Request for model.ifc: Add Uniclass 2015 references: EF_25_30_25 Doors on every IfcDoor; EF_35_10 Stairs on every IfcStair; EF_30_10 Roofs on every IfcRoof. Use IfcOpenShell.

First a look at what the model holds.

```python
import ifcopenshell

model = ifcopenshell.open("model.ifc")
print(model.schema)
print("classifications:", [c.Name for c in model.by_type("IfcClassification")])
for ifc_class in ("IfcDoor", "IfcRoof", "IfcStair", "IfcWall", "IfcWindow"):
    print(ifc_class, len(model.by_type(ifc_class)))
```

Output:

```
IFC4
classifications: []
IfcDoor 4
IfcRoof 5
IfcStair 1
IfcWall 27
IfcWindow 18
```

```python
import ifcopenshell
import ifcopenshell.api.classification

model = ifcopenshell.open("model.ifc")

system = ifcopenshell.api.classification.add_classification(model, classification="Uniclass 2015")

codes = {
    "IfcDoor": ("EF_25_30_25", "Doors"),
    "IfcStair": ("EF_35_10", "Stairs"),
    "IfcRoof": ("EF_30_10", "Roofs"),
}
for ifc_class, (code, name) in codes.items():
    products = model.by_type(ifc_class)
    ifcopenshell.api.classification.add_reference(
        model, products=products, classification=system, identification=code, name=name
    )
    print(code, len(products))

model.write("model_v2.ifc")
```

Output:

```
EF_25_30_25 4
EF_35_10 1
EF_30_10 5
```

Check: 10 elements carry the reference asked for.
